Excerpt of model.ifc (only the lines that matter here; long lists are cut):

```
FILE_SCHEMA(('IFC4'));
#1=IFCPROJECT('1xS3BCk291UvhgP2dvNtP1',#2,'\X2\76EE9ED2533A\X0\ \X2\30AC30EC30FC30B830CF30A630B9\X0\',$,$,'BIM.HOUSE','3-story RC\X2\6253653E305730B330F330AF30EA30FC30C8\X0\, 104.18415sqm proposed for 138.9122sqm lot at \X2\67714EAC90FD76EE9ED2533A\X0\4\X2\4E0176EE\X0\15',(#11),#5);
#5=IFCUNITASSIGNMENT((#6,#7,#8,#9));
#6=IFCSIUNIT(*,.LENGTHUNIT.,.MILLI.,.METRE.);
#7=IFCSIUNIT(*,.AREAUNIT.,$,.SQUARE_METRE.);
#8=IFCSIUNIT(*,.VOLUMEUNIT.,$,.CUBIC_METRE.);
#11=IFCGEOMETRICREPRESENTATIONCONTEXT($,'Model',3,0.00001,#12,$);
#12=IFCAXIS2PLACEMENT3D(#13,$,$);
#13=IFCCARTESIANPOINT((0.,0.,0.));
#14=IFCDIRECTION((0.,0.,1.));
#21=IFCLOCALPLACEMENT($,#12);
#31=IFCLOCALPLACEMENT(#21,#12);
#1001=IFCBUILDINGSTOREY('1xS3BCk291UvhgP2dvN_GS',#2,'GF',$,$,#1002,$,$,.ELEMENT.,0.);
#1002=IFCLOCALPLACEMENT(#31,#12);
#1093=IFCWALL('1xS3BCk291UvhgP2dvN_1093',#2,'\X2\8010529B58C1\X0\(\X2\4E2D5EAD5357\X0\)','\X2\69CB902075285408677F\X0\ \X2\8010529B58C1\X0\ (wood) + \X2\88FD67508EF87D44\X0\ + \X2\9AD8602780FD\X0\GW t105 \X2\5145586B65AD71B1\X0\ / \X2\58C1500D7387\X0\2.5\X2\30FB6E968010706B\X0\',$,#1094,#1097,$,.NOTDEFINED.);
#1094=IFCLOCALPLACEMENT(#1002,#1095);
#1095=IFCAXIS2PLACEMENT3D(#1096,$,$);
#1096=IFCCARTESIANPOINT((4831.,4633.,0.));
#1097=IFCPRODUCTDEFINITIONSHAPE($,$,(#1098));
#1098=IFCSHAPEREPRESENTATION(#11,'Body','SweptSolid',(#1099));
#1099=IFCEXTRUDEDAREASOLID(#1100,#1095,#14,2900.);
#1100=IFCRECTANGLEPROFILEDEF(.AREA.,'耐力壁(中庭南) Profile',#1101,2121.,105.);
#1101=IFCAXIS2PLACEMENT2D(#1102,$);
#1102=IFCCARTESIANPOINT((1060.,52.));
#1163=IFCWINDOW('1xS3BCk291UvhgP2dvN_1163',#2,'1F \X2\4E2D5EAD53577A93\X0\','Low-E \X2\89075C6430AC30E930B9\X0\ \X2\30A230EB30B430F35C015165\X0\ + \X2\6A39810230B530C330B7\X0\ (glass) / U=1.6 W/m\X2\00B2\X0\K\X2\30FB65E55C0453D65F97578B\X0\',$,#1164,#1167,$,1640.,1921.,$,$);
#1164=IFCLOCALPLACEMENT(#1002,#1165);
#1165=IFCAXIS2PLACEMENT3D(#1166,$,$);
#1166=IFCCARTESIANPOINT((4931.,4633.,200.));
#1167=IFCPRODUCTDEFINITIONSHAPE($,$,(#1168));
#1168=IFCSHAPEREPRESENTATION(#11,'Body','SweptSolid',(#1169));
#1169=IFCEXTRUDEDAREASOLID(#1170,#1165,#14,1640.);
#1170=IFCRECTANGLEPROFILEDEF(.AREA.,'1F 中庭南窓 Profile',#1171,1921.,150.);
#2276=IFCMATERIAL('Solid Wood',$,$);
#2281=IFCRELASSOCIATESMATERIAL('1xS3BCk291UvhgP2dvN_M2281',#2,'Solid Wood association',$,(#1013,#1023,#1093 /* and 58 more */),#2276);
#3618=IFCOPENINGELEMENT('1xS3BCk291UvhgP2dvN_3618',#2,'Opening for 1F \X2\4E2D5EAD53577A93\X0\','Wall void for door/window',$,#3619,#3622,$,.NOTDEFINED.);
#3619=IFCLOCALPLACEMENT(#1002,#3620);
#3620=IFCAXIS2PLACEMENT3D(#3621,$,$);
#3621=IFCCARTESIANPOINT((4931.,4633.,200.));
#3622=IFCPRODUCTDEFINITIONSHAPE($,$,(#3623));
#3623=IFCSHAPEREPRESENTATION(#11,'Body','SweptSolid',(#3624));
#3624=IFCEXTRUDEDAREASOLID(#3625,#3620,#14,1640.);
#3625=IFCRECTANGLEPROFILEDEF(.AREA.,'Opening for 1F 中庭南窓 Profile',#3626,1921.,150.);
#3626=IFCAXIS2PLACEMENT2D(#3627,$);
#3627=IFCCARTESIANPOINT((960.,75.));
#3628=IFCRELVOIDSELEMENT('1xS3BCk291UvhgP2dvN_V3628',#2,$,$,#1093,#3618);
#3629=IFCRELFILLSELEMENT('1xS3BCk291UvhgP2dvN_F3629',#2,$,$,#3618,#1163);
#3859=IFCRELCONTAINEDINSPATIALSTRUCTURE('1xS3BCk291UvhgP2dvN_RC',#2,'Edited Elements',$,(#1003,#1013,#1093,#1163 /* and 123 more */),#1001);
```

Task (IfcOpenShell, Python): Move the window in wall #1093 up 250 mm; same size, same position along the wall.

```python
import numpy as np
import ifcopenshell
import ifcopenshell.api.geometry
import ifcopenshell.util.placement
import ifcopenshell.util.unit

model = ifcopenshell.open("model.ifc")
unit_scale = ifcopenshell.util.unit.calculate_unit_scale(model)

window = model.by_guid("1xS3BCk291UvhgP2dvN_1163")
opening = window.FillsVoids[0].RelatingOpeningElement
dz = 0.25 / unit_scale

shift = np.array([0.0, 0.0, dz])
# The window is not placed relative to its opening, so move both.
for product in (opening, window):
    matrix = ifcopenshell.util.placement.get_local_placement(product.ObjectPlacement)
    matrix[:3, 3] += shift
    ifcopenshell.api.geometry.edit_object_placement(model, product=product, matrix=matrix, is_si=False)

print(f"moved by {dz * unit_scale:+.3f} m")

model.write("model_v2.ifc")
```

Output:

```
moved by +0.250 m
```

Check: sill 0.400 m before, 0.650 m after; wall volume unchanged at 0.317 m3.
